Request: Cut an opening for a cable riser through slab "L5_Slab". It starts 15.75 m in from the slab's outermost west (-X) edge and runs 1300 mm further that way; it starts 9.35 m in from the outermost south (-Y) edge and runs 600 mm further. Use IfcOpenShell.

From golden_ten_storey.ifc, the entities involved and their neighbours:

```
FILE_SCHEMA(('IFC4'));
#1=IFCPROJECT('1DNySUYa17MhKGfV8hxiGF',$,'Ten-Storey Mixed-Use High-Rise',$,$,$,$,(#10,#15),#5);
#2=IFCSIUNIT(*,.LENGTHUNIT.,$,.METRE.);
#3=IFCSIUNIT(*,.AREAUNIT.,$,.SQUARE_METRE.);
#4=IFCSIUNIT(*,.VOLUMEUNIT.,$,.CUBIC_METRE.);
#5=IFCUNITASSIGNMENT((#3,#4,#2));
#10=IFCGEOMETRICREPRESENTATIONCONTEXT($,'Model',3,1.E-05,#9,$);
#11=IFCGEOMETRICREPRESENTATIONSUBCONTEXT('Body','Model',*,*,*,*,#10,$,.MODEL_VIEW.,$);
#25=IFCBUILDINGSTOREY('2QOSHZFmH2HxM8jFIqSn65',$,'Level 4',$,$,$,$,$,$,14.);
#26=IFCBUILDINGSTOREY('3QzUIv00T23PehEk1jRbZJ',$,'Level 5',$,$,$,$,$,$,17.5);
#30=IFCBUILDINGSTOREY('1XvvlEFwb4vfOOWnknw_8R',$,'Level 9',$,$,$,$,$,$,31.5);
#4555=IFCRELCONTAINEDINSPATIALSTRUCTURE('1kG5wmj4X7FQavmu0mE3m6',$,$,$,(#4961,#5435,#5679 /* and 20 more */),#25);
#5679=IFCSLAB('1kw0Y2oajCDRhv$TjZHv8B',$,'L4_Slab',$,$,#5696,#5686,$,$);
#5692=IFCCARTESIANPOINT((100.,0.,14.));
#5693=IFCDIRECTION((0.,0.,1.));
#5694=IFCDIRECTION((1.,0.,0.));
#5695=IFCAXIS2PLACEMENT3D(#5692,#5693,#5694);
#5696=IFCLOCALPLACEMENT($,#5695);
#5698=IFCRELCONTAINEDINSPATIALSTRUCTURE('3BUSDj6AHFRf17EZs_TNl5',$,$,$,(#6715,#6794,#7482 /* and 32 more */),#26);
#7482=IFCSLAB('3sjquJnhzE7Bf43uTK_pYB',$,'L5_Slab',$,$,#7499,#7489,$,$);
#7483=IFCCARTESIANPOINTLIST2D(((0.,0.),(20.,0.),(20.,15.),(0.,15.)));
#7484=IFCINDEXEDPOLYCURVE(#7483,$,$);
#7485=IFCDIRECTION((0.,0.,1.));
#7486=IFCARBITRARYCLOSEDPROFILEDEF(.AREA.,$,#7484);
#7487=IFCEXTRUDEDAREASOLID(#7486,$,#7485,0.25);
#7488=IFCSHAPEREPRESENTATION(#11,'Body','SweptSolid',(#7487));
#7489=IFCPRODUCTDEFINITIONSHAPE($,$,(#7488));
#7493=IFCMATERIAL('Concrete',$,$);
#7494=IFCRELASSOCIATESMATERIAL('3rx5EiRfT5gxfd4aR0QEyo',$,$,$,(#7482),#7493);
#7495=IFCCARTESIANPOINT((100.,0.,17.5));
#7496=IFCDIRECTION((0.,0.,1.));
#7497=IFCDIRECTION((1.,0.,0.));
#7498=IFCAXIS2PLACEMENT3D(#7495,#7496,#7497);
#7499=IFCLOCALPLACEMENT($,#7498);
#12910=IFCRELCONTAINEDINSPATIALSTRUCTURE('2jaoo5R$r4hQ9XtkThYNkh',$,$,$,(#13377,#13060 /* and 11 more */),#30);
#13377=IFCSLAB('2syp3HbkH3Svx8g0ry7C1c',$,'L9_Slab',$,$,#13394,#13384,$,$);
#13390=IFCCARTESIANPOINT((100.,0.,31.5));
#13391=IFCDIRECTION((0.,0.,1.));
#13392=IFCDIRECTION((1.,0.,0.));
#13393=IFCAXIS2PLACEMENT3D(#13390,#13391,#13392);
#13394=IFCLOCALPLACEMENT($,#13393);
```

```python
import numpy as np
import ifcopenshell
import ifcopenshell.api.feature
import ifcopenshell.api.geometry
import ifcopenshell.api.root
import ifcopenshell.geom
import ifcopenshell.util.placement
import ifcopenshell.util.representation
import ifcopenshell.util.shape
import ifcopenshell.util.unit

model = ifcopenshell.open("golden_ten_storey.ifc")
unit_scale = ifcopenshell.util.unit.calculate_unit_scale(model)
settings = ifcopenshell.geom.settings()


def volume(element):
    """Net volume in cubic metres, openings subtracted."""
    shape = ifcopenshell.geom.create_shape(settings, element)
    return ifcopenshell.util.shape.get_volume(shape.geometry)


slab = model.by_guid("3sjquJnhzE7Bf43uTK_pYB")
before = volume(slab)

# Extent in the slab's own axes, in metres. The edges named are its -X and -Y sides.
slab_shape = ifcopenshell.geom.create_shape(settings, slab)
vertices = ifcopenshell.util.shape.get_vertices(slab_shape.geometry)
x_min, y_min, bottom = vertices.min(axis=0)
top = vertices[:, 2].max()

opening = ifcopenshell.api.root.create_entity(model, ifc_class="IfcOpeningElement", name="Cable riser opening", predefined_type="OPENING")
context = ifcopenshell.util.representation.get_context(model, "Model", "Body", "MODEL_VIEW")
width, depth = 1.3, 0.6
outline = [(0.0, 0.0), (width, 0.0), (width, depth), (0.0, depth), (0.0, 0.0)]
# Overshoot both faces by 50 mm so the cut is clean.
shape = ifcopenshell.api.geometry.add_slab_representation(
    model, context=context, depth=top - bottom + 0.1, polyline=outline
)
ifcopenshell.api.geometry.assign_representation(model, product=opening, representation=shape)

matrix = ifcopenshell.util.placement.get_local_placement(slab.ObjectPlacement)
matrix[:, 3] = matrix @ np.append(np.array([x_min + 15.75, y_min + 9.35, bottom - 0.05]) / unit_scale, 1.0)
ifcopenshell.api.geometry.edit_object_placement(model, product=opening, matrix=matrix, is_si=False)
ifcopenshell.api.feature.add_feature(model, feature=opening, element=slab)

after = volume(slab)

print(f"slab volume {before:.3f} -> {after:.3f} m3")

model.write("golden_ten_storey_v2.ifc")
```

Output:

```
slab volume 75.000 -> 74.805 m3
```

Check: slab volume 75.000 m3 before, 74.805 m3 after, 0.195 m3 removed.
